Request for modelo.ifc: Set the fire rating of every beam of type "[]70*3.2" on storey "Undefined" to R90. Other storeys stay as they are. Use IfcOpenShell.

First a look at what the model holds.

```python
import ifcopenshell
import ifcopenshell.util.element

model = ifcopenshell.open("modelo.ifc")
print(model.schema)
storey = next(s for s in model.by_type("IfcBuildingStorey") if s.Name == "Undefined")
beams = [e for e in ifcopenshell.util.element.get_decomposition(storey) if e.is_a("IfcBeam")]
seen = {}
for e in beams:
    element_type = ifcopenshell.util.element.get_type(e)
    key = (element_type.Name if element_type != e and element_type else None, ifcopenshell.util.element.get_pset(e, "Pset_BeamCommon", "FireRating"))
    seen[key] = seen.get(key, 0) + 1
for (name, value), count in sorted(seen.items(), key=str):
    print(count, "x", name, "|", value)
```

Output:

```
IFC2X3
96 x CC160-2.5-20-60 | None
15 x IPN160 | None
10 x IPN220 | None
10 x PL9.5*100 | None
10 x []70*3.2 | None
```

```python
import ifcopenshell
import ifcopenshell.api.pset
import ifcopenshell.util.element

model = ifcopenshell.open("modelo.ifc")

storey = next(s for s in model.by_type("IfcBuildingStorey") if s.Name == "Undefined")
beams = [e for e in ifcopenshell.util.element.get_decomposition(storey) if e.is_a("IfcBeam")]

count = 0
for e in beams:
    element_type = ifcopenshell.util.element.get_type(e)
    if element_type in (None, e) or element_type.Name != "[]70*3.2":
        continue
    found = ifcopenshell.util.element.get_pset(e, "Pset_BeamCommon", should_inherit=False)
    if found:
        pset = model.by_id(found["id"])
        if len(ifcopenshell.util.element.get_elements_by_pset(pset)) > 1:
            pset = ifcopenshell.api.pset.unshare_pset(model, products=[e], pset=pset)[0]
    else:
        pset = ifcopenshell.api.pset.add_pset(model, product=e, name="Pset_BeamCommon")
    ifcopenshell.api.pset.edit_pset(model, pset=pset, properties={"FireRating": "R90"})
    count += 1

print(count, "beams updated")

model.write("modelo_edited.ifc")
```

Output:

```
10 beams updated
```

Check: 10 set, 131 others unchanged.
